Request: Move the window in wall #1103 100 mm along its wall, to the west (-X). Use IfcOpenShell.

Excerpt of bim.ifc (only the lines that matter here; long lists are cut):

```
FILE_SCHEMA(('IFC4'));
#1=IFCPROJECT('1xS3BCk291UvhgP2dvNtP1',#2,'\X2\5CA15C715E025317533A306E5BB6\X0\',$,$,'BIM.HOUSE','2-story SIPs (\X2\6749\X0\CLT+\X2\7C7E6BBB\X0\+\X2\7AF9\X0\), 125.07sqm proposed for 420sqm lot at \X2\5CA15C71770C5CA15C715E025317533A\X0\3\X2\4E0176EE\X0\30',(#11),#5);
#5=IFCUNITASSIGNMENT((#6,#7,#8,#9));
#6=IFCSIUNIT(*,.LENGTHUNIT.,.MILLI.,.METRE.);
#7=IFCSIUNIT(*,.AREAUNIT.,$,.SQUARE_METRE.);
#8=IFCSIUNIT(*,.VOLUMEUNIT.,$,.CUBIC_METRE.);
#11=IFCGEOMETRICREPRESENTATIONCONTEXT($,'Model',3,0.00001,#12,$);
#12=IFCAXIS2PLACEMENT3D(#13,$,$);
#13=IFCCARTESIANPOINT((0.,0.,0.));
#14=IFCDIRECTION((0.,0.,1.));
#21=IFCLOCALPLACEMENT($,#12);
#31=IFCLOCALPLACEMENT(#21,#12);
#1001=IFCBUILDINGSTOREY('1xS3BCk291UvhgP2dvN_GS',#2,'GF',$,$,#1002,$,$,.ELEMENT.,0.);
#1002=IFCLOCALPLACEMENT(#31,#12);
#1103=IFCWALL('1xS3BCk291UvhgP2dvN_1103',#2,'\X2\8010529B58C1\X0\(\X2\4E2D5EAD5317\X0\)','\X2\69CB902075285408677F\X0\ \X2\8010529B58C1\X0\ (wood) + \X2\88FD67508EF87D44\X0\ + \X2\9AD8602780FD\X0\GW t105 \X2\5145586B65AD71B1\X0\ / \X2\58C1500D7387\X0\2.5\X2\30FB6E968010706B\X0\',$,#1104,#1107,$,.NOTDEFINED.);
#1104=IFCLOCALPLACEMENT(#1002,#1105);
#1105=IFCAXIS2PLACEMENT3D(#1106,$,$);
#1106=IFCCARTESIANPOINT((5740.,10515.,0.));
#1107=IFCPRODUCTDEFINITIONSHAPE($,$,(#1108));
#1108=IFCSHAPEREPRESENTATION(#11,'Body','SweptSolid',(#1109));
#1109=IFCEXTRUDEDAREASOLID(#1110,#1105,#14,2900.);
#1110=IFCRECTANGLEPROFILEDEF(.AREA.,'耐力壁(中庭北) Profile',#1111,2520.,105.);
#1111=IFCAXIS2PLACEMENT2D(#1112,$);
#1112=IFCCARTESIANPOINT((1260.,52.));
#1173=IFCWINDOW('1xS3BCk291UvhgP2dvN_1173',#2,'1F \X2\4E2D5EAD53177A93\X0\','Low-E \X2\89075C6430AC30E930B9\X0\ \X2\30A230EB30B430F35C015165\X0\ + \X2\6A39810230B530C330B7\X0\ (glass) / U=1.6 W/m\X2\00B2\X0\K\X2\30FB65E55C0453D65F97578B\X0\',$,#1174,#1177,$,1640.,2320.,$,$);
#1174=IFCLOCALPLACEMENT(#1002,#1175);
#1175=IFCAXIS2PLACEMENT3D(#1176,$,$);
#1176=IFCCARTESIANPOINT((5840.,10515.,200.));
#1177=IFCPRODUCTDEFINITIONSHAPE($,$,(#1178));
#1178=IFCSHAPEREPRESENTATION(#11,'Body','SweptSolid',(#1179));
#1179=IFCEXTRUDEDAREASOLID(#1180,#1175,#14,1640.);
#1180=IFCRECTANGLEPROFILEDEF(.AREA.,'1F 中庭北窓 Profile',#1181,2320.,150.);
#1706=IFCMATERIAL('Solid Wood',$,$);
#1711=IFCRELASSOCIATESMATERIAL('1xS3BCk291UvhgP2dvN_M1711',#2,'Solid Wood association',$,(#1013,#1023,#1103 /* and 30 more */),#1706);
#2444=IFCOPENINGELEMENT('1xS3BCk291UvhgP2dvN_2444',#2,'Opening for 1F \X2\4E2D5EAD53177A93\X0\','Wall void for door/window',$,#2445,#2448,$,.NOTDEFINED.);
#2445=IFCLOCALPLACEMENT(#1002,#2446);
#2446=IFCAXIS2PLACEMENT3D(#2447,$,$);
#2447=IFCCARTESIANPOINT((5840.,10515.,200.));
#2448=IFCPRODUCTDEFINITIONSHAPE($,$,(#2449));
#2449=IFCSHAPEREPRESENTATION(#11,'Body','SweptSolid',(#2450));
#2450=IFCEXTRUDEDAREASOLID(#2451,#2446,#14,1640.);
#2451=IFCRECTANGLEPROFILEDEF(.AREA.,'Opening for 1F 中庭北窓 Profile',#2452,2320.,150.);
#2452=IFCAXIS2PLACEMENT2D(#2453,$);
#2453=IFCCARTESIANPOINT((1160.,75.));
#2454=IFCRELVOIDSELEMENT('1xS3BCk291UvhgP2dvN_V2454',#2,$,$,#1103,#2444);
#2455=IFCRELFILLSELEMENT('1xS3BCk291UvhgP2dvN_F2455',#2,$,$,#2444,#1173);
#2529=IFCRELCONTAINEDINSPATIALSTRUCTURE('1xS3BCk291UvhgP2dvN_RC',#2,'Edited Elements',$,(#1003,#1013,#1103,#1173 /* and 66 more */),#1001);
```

```python
import ifcopenshell
import ifcopenshell.api.geometry
import ifcopenshell.util.placement
import ifcopenshell.util.unit

model = ifcopenshell.open("bim.ifc")
unit_scale = ifcopenshell.util.unit.calculate_unit_scale(model)

window = model.by_id(1173)
opening = window.FillsVoids[0].RelatingOpeningElement
wall = opening.VoidsElements[0].RelatingBuildingElement

wall_matrix = ifcopenshell.util.placement.get_local_placement(wall.ObjectPlacement)
shift = wall_matrix[:3, 0] * -0.1 / unit_scale
before = ifcopenshell.util.placement.get_local_placement(window.ObjectPlacement)[:3, 3].copy()

# The window is not placed relative to its opening, so move both.
for product in (opening, window):
    matrix = ifcopenshell.util.placement.get_local_placement(product.ObjectPlacement)
    matrix[:3, 3] += shift
    ifcopenshell.api.geometry.edit_object_placement(model, product=product, matrix=matrix, is_si=False)

after = ifcopenshell.util.placement.get_local_placement(window.ObjectPlacement)[:3, 3]
print("window moved by", (after - before).round(3) + 0.0)

model.write("bim_v2.ifc")
```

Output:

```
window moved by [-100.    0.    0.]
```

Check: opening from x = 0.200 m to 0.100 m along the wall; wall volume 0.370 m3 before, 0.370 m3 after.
